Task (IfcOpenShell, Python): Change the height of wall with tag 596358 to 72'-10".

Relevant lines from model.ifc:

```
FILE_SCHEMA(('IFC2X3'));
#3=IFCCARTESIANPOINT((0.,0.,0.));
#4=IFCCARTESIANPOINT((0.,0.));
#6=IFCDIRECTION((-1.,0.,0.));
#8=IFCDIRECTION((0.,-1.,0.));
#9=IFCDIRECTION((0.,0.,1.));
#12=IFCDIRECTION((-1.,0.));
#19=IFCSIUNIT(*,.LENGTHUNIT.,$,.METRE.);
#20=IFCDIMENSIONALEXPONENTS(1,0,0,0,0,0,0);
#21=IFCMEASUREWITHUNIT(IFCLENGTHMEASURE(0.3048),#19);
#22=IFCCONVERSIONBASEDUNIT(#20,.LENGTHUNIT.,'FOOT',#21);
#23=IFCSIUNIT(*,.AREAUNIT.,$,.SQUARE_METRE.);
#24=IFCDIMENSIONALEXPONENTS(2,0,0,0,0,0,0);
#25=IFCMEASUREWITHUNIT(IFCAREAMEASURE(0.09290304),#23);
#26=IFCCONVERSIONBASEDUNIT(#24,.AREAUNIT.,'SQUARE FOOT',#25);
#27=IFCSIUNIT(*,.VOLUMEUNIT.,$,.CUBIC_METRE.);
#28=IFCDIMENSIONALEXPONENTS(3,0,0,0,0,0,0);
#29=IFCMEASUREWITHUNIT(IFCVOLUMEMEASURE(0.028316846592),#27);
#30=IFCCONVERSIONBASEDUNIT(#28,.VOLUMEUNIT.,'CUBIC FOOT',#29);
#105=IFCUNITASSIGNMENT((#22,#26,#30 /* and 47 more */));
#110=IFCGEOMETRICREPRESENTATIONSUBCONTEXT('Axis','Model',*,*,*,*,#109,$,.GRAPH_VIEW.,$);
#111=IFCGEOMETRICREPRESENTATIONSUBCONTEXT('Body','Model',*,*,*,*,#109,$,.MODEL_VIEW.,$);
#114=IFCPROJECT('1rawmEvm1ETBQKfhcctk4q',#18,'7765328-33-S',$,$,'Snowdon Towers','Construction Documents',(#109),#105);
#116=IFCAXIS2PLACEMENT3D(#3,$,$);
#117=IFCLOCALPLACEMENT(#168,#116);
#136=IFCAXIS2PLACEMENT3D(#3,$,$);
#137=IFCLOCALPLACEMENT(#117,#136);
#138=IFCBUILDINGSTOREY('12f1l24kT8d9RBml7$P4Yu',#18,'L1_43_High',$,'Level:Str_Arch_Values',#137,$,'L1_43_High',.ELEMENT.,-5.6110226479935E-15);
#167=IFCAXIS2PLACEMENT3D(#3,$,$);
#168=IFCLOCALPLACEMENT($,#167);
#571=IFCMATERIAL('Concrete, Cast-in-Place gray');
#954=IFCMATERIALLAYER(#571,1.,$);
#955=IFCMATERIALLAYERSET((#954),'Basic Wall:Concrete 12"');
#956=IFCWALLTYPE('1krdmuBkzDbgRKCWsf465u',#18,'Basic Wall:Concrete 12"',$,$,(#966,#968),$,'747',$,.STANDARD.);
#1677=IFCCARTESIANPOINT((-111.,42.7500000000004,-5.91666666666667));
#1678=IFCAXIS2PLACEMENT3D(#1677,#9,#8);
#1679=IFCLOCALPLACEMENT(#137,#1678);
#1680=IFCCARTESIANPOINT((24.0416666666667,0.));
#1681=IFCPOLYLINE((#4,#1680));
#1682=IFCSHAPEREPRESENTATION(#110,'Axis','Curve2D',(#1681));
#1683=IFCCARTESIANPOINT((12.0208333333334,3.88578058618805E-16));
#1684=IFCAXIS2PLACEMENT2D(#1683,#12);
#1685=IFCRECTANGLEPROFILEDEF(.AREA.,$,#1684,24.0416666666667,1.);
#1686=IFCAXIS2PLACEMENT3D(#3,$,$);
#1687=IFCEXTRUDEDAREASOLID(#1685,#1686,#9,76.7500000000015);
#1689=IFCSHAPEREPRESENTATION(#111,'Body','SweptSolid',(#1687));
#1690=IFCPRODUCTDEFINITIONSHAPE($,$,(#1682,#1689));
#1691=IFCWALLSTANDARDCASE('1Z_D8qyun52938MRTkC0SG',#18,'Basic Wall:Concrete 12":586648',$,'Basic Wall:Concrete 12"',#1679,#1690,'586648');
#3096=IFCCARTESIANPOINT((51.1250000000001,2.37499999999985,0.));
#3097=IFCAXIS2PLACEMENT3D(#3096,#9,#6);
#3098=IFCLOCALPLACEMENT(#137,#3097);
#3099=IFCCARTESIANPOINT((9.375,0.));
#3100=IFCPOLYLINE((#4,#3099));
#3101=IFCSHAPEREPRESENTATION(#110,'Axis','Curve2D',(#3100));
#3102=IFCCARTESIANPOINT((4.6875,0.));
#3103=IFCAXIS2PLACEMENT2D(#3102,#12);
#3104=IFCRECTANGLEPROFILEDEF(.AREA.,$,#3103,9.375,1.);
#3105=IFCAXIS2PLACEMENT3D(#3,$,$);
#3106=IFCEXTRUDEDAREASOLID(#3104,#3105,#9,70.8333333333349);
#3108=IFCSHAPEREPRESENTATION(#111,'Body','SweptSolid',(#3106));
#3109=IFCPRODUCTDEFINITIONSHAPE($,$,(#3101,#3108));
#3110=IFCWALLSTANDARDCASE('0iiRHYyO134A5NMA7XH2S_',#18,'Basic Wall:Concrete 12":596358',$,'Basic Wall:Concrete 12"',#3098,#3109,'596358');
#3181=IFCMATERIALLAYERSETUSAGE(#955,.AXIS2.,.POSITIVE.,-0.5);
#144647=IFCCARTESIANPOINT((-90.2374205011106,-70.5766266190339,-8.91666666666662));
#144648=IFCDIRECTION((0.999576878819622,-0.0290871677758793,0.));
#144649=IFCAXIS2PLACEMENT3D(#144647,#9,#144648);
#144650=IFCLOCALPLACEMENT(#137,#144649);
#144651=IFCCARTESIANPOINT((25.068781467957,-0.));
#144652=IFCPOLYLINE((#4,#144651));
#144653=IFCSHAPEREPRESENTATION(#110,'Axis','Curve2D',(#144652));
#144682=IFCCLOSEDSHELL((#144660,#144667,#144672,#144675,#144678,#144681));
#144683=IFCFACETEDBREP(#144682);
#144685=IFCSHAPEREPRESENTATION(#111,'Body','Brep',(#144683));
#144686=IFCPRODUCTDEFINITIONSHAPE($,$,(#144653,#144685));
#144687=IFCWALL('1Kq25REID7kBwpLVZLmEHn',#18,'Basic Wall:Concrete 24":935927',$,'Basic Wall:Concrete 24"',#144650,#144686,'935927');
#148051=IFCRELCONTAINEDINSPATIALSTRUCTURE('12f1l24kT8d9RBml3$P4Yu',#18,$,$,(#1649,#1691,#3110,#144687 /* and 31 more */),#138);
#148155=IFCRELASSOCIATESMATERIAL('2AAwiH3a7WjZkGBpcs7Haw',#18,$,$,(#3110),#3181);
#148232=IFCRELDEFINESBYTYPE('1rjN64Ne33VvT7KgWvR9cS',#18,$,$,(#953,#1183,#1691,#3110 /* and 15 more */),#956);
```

```python
import ifcopenshell
import ifcopenshell.geom
import ifcopenshell.util.representation
import ifcopenshell.util.shape
import ifcopenshell.util.unit

model = ifcopenshell.open("model.ifc")
unit_scale = ifcopenshell.util.unit.calculate_unit_scale(model)
settings = ifcopenshell.geom.settings()


def volume(element):
    """Net volume in cubic metres, openings subtracted."""
    shape = ifcopenshell.geom.create_shape(settings, element)
    return ifcopenshell.util.shape.get_volume(shape.geometry)


wall = model.by_guid("0iiRHYyO134A5NMA7XH2S_")
before = volume(wall)

body = ifcopenshell.util.representation.get_representation(wall, "Model", "Body")
solid = body.Items[0]
old_height = solid.Depth
solid.Depth = 874 * 0.0254 / unit_scale
after = volume(wall)

print(f"height {old_height:g} -> {solid.Depth:g}, volume {before:.3f} -> {after:.3f} m3")

model.write("model_v2.ifc")
```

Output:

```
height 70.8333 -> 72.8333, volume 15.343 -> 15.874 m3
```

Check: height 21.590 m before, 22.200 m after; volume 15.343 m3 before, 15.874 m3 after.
